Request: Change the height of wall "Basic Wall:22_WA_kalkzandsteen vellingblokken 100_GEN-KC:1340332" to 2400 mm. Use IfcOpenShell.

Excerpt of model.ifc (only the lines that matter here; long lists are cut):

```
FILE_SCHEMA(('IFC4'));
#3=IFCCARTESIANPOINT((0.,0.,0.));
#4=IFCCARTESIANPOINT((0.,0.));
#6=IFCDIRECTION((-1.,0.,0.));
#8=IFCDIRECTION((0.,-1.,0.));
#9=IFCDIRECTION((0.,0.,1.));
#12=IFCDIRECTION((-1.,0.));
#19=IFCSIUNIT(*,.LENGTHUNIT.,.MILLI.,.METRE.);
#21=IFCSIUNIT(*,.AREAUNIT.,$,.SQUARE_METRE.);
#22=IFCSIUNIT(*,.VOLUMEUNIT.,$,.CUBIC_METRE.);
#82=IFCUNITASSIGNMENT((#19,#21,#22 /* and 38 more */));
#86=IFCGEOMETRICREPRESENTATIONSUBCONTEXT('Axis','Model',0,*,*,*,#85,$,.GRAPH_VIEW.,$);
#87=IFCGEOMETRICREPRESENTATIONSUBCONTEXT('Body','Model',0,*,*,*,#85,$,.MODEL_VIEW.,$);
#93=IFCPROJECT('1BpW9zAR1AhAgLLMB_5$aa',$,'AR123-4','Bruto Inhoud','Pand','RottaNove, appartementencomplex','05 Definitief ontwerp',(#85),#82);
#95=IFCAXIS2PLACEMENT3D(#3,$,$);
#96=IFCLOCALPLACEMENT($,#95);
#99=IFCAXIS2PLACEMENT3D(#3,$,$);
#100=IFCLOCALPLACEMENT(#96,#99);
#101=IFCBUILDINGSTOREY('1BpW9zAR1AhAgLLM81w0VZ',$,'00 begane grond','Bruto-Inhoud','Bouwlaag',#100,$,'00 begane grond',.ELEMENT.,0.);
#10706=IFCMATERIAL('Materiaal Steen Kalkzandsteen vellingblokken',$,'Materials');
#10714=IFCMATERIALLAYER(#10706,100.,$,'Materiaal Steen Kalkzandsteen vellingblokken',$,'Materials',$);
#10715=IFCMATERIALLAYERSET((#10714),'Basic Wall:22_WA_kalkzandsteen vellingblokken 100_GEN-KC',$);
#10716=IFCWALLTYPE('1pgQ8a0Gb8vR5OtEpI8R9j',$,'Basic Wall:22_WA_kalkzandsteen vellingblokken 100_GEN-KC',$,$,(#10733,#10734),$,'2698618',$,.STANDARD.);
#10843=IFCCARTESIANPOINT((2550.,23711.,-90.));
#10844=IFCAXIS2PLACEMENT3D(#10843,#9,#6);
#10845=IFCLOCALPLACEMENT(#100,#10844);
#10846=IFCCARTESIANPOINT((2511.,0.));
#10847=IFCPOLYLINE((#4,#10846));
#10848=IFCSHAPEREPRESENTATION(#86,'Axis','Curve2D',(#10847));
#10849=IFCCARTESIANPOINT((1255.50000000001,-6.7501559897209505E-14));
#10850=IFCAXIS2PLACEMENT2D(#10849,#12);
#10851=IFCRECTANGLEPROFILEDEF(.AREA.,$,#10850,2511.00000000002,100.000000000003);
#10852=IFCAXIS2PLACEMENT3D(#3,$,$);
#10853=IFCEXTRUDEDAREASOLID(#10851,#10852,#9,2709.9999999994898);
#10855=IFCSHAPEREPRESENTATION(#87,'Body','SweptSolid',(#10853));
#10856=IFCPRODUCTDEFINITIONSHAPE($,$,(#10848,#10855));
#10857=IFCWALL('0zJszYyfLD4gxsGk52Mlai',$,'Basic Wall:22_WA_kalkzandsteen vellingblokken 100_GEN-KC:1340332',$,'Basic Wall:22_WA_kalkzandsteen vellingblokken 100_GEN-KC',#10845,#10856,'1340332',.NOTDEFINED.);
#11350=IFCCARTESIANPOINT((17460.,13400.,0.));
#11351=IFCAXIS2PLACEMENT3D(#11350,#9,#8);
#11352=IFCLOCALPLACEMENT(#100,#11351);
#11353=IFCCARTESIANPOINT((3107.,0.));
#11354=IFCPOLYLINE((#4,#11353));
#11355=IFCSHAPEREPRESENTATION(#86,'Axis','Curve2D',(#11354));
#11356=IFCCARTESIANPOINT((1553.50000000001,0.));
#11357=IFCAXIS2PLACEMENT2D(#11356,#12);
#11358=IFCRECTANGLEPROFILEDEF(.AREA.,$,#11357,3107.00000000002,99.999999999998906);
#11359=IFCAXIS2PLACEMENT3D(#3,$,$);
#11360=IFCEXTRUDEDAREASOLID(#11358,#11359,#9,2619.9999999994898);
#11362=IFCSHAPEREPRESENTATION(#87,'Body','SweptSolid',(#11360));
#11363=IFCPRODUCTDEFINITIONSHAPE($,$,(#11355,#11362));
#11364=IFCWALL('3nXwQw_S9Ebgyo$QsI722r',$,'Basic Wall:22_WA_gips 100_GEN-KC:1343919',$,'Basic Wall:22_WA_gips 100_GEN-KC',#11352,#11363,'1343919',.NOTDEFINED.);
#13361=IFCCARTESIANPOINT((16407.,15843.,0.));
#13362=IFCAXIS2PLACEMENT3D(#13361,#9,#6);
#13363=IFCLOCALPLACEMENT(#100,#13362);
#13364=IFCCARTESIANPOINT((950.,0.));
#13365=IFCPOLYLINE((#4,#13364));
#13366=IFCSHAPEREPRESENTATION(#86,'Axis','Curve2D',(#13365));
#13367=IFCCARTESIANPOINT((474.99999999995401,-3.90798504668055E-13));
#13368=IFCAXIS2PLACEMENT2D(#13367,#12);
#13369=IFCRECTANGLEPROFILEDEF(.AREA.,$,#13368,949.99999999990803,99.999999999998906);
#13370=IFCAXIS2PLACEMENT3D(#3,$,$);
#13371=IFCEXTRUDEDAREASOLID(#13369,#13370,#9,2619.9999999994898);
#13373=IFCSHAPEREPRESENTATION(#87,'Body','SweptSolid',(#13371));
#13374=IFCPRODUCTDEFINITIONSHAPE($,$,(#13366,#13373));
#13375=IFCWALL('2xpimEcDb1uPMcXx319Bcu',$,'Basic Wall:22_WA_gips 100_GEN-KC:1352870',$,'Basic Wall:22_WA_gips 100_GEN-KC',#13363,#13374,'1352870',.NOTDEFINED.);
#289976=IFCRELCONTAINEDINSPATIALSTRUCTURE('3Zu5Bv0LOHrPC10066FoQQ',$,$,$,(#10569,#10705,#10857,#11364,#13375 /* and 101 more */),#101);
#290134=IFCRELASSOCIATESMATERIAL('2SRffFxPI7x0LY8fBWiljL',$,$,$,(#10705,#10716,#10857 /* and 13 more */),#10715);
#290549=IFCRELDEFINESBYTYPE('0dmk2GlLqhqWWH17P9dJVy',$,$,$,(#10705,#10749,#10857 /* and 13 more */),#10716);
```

```python
import ifcopenshell
import ifcopenshell.geom
import ifcopenshell.util.representation
import ifcopenshell.util.shape

model = ifcopenshell.open("model.ifc")
settings = ifcopenshell.geom.settings()


def volume(element):
    """Net volume in cubic metres, openings subtracted."""
    shape = ifcopenshell.geom.create_shape(settings, element)
    return ifcopenshell.util.shape.get_volume(shape.geometry)


wall = model.by_guid("0zJszYyfLD4gxsGk52Mlai")
before = volume(wall)

body = ifcopenshell.util.representation.get_representation(wall, "Model", "Body")
solid = body.Items[0]
old_height = solid.Depth
solid.Depth = 2400.0
after = volume(wall)

print(f"height {old_height:g} -> {solid.Depth:g}, volume {before:.3f} -> {after:.3f} m3")

model.write("model_v2.ifc")
```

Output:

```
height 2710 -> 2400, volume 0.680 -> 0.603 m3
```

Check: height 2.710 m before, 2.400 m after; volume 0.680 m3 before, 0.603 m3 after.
